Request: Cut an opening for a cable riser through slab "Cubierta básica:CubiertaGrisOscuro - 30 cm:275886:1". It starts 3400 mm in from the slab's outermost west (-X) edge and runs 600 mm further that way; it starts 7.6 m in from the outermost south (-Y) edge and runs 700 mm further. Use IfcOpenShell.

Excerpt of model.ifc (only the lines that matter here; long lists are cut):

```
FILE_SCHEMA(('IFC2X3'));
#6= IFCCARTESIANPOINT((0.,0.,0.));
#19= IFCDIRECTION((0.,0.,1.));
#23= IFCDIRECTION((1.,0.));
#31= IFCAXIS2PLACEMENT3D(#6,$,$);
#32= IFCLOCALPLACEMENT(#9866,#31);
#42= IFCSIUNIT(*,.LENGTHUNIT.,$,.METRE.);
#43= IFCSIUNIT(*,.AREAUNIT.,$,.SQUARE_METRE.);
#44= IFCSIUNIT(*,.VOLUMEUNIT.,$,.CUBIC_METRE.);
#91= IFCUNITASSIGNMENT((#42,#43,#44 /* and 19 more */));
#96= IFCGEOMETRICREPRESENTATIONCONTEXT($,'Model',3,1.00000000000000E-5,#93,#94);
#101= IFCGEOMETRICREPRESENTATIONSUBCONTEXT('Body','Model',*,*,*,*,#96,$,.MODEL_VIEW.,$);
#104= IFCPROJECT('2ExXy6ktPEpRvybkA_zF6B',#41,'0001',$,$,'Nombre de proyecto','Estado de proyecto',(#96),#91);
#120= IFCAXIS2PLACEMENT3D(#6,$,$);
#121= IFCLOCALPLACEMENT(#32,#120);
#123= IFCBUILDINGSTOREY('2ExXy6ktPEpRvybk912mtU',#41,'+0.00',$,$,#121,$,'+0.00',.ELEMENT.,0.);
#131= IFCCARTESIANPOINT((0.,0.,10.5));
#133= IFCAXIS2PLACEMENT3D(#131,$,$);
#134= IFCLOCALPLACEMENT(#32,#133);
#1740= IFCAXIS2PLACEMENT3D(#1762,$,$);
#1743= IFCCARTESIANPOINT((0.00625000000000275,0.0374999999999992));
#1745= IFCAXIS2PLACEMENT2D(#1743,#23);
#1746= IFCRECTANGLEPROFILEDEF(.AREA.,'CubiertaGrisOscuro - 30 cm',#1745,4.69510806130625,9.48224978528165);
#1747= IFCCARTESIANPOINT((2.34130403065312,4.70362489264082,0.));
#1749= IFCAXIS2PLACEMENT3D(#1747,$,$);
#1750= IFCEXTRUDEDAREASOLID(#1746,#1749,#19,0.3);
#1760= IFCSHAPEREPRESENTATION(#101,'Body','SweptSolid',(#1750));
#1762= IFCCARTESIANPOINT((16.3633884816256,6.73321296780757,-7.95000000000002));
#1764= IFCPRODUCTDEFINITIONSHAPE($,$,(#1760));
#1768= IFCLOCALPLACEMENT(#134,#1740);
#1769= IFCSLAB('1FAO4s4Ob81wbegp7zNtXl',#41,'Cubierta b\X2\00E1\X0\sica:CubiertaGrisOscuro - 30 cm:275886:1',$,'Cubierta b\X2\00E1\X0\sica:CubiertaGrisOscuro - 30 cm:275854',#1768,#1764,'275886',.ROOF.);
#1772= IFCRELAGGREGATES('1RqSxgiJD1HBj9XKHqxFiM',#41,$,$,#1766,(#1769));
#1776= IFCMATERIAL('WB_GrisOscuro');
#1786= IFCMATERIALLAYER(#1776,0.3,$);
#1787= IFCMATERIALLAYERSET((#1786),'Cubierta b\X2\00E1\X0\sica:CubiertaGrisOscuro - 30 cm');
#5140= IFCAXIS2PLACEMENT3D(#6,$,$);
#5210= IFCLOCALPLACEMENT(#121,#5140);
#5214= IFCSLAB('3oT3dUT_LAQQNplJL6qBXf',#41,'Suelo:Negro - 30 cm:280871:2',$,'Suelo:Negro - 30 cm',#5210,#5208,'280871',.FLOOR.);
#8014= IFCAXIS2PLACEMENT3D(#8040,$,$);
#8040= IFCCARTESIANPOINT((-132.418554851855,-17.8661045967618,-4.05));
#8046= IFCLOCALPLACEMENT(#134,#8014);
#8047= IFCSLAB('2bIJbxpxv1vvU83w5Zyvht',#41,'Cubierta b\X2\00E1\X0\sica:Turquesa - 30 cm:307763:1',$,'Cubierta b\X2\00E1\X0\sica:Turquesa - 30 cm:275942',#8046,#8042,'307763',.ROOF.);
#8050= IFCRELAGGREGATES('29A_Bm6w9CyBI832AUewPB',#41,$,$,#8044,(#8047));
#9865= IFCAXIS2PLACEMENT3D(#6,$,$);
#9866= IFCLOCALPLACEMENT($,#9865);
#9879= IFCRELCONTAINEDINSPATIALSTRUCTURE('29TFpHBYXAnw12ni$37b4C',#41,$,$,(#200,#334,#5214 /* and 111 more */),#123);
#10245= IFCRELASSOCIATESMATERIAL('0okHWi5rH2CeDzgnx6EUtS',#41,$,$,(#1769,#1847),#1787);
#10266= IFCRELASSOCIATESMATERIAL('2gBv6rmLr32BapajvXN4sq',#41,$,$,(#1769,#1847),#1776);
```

```python
import numpy as np
import ifcopenshell
import ifcopenshell.api.feature
import ifcopenshell.api.geometry
import ifcopenshell.api.root
import ifcopenshell.geom
import ifcopenshell.util.placement
import ifcopenshell.util.representation
import ifcopenshell.util.shape
import ifcopenshell.util.unit

model = ifcopenshell.open("model.ifc")
unit_scale = ifcopenshell.util.unit.calculate_unit_scale(model)
settings = ifcopenshell.geom.settings()


def volume(element):
    """Net volume in cubic metres, openings subtracted."""
    shape = ifcopenshell.geom.create_shape(settings, element)
    return ifcopenshell.util.shape.get_volume(shape.geometry)


slab = model.by_guid("1FAO4s4Ob81wbegp7zNtXl")
before = volume(slab)

# Extent in the slab's own axes, in metres. The edges named are its -X and -Y sides.
slab_shape = ifcopenshell.geom.create_shape(settings, slab)
vertices = ifcopenshell.util.shape.get_vertices(slab_shape.geometry)
x_min, y_min, bottom = vertices.min(axis=0)
top = vertices[:, 2].max()

opening = ifcopenshell.api.root.create_entity(model, ifc_class="IfcOpeningElement", name="Cable riser opening")
context = ifcopenshell.util.representation.get_context(model, "Model", "Body", "MODEL_VIEW")
width, depth = 0.6, 0.7
outline = [(0.0, 0.0), (width, 0.0), (width, depth), (0.0, depth), (0.0, 0.0)]
# Overshoot both faces by 50 mm so the cut is clean.
shape = ifcopenshell.api.geometry.add_slab_representation(
    model, context=context, depth=top - bottom + 0.1, polyline=outline
)
ifcopenshell.api.geometry.assign_representation(model, product=opening, representation=shape)

matrix = ifcopenshell.util.placement.get_local_placement(slab.ObjectPlacement)
matrix[:, 3] = matrix @ np.append(np.array([x_min + 3.4, y_min + 7.6, bottom - 0.05]) / unit_scale, 1.0)
ifcopenshell.api.geometry.edit_object_placement(model, product=opening, matrix=matrix, is_si=False)
ifcopenshell.api.feature.add_feature(model, feature=opening, element=slab)

after = volume(slab)

print(f"slab volume {before:.3f} -> {after:.3f} m3")

model.write("model_edited.ifc")
```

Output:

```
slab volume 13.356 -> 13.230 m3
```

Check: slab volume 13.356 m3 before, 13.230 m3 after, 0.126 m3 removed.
